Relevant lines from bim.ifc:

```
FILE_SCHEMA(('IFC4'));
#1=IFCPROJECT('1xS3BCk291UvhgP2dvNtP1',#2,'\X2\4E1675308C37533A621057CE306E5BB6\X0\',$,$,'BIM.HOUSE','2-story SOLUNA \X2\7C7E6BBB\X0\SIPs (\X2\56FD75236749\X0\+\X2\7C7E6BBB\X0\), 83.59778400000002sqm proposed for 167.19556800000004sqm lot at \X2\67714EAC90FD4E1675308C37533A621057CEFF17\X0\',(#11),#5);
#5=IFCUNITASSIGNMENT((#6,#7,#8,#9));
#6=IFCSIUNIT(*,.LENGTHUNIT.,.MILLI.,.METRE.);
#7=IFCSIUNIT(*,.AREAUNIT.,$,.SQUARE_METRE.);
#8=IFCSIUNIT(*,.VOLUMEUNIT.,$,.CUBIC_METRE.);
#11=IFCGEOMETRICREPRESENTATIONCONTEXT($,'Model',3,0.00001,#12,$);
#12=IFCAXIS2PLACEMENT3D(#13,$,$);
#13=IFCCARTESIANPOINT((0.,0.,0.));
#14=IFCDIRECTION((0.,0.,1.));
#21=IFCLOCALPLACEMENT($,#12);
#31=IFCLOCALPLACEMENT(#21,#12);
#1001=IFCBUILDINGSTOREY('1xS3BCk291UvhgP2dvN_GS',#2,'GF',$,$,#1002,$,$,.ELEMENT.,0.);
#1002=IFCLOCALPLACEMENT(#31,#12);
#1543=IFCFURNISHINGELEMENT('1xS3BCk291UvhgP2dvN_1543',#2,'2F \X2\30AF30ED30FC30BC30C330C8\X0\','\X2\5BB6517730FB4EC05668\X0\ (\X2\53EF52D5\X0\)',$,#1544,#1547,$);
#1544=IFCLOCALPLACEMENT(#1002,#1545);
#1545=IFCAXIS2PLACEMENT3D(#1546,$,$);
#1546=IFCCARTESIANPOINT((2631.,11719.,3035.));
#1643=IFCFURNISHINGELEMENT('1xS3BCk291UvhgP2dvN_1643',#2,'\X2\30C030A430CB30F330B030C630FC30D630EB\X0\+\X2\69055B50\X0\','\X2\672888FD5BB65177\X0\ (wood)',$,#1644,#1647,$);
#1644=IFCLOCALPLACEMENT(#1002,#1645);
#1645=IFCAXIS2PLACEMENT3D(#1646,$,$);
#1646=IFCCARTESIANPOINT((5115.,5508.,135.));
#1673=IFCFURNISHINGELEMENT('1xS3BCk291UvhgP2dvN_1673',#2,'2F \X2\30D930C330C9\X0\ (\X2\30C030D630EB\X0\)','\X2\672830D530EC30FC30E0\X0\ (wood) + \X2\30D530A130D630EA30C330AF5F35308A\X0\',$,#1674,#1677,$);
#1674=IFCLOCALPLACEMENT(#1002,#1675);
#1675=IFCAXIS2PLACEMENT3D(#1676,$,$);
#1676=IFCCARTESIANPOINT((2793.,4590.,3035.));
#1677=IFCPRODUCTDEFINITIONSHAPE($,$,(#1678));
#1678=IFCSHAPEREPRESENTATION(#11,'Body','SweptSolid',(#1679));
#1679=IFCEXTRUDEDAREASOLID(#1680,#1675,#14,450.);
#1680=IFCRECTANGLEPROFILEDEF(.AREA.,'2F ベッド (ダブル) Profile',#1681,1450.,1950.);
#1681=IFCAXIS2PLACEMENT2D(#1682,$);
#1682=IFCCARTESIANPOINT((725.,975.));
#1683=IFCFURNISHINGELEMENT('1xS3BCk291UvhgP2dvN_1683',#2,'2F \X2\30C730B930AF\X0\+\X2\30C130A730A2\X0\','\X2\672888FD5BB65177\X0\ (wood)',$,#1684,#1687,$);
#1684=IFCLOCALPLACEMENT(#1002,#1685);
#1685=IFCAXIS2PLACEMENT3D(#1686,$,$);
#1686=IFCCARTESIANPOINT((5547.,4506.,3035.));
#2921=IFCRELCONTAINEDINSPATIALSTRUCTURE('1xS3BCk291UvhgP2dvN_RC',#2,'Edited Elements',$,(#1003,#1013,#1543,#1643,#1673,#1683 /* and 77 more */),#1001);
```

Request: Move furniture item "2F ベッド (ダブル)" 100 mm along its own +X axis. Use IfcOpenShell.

```python
import ifcopenshell
import ifcopenshell.api.geometry
import ifcopenshell.util.placement

model = ifcopenshell.open("bim.ifc")

item = model.by_id(1673)
matrix = ifcopenshell.util.placement.get_local_placement(item.ObjectPlacement)
matrix[:3, 3] += matrix[:3, 0] * 100.0
ifcopenshell.api.geometry.edit_object_placement(model, product=item, matrix=matrix, is_si=False)

print(ifcopenshell.util.placement.get_local_placement(item.ObjectPlacement).round(3) + 0.0)

model.write("bim_edited.ifc")
```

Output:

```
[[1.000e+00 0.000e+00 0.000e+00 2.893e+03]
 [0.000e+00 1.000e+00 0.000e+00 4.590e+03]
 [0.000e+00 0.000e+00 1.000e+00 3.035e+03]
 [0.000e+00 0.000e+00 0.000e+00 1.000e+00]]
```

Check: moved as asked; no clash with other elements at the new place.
